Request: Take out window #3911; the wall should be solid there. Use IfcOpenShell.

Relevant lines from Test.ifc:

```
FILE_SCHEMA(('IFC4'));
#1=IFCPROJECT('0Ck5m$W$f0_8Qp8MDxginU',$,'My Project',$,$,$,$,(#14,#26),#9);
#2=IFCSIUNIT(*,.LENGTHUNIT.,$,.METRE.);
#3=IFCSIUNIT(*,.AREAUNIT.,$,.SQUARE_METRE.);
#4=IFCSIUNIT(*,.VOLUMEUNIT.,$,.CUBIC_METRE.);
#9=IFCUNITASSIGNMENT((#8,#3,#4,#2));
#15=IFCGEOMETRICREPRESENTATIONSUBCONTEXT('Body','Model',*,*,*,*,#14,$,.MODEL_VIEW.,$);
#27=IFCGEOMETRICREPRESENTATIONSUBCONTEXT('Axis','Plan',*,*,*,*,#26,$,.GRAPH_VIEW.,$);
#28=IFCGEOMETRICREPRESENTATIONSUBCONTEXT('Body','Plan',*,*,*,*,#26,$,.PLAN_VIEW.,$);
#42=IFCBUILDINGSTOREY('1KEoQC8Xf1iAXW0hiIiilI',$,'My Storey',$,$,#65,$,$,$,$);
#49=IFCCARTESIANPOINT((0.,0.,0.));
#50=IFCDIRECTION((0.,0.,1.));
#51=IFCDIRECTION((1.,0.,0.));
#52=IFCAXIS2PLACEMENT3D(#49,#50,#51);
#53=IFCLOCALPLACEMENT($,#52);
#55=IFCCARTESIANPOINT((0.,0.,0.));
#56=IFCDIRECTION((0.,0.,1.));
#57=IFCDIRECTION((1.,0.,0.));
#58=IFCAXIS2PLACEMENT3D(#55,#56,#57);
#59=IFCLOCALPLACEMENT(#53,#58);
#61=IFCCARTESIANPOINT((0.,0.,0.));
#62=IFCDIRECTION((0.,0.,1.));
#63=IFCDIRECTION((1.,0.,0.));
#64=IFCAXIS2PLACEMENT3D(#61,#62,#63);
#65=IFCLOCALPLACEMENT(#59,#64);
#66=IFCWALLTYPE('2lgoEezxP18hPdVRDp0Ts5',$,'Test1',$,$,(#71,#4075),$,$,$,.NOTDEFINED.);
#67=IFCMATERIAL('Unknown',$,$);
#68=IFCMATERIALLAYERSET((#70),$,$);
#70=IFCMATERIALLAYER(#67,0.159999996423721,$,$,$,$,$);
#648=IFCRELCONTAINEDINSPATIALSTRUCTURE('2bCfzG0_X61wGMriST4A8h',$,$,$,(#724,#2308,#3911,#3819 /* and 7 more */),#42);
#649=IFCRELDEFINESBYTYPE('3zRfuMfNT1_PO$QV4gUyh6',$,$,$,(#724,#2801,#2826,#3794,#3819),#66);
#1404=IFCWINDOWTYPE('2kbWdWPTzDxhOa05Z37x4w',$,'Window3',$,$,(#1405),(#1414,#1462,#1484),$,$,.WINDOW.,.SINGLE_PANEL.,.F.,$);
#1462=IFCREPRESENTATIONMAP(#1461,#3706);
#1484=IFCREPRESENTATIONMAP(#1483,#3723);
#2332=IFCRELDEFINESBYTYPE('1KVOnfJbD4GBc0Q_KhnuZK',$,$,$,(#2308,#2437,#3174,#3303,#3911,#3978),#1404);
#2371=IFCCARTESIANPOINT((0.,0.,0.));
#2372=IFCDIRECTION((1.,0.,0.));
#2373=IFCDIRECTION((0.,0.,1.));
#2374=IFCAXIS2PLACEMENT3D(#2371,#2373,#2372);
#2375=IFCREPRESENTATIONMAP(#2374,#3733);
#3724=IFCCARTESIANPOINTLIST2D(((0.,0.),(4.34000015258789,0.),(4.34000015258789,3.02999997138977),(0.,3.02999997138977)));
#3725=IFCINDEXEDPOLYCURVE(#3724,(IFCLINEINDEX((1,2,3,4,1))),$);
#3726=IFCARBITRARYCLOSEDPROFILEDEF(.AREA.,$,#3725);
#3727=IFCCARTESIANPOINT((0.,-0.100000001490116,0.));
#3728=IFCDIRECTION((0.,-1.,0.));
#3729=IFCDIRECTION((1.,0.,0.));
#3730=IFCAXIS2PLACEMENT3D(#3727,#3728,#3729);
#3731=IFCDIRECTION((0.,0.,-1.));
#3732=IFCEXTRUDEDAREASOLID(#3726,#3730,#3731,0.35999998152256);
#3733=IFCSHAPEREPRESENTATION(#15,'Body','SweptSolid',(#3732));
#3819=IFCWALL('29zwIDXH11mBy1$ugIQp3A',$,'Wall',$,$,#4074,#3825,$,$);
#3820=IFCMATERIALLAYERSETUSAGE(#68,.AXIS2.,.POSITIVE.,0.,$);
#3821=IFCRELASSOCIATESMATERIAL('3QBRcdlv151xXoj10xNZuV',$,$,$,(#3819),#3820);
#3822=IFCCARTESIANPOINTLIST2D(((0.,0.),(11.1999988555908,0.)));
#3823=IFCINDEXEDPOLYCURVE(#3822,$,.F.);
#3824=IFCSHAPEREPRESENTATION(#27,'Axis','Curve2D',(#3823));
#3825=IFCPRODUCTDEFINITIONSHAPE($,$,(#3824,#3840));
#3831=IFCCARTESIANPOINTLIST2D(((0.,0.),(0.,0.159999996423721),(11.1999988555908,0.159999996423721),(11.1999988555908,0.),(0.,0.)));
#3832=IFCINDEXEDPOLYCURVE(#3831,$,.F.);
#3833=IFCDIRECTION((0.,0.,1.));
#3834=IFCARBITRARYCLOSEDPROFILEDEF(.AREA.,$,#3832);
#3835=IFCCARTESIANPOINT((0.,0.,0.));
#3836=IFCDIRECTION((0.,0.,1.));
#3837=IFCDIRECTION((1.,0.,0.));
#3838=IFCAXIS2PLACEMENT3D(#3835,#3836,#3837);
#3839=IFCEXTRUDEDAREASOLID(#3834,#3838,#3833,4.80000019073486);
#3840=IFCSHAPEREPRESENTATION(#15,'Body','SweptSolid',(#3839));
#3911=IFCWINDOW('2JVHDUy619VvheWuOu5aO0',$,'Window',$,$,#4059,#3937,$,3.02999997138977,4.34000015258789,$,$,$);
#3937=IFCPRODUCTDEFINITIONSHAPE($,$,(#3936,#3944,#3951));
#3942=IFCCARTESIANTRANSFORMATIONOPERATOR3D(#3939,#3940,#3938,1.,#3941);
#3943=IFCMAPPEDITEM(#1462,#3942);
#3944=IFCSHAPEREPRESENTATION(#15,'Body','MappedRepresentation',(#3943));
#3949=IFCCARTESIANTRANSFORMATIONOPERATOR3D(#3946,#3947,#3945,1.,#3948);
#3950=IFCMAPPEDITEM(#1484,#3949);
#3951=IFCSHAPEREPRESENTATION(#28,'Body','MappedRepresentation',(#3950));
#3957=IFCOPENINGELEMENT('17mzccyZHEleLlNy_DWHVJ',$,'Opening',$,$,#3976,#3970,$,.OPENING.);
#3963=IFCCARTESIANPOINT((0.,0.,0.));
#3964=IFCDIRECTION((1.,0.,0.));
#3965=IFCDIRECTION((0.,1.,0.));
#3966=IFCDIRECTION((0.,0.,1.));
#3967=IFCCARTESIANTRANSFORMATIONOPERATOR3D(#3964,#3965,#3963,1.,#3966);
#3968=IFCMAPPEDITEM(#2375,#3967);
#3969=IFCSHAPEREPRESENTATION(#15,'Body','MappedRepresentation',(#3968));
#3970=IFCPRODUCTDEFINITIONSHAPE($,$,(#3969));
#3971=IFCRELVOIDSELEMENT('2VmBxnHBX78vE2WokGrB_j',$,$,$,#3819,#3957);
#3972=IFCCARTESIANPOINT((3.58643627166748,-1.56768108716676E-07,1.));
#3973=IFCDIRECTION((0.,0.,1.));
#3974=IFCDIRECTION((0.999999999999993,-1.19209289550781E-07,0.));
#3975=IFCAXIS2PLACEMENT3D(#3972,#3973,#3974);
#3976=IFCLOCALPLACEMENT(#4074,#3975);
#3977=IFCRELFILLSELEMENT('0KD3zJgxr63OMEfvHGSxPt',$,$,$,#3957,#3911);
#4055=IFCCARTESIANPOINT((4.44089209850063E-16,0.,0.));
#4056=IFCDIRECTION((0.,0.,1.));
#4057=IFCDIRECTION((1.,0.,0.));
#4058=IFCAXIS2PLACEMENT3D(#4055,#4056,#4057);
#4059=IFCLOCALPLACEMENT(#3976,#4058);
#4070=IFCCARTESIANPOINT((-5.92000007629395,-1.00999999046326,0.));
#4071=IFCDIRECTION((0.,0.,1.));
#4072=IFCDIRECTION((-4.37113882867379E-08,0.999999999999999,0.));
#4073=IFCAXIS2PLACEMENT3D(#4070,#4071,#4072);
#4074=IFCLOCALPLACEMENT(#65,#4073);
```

```python
import ifcopenshell
import ifcopenshell.api.feature
import ifcopenshell.api.root
import ifcopenshell.geom
import ifcopenshell.util.shape

model = ifcopenshell.open("Test.ifc")
settings = ifcopenshell.geom.settings()


def volume(element):
    """Net volume in cubic metres, openings subtracted."""
    shape = ifcopenshell.geom.create_shape(settings, element)
    return ifcopenshell.util.shape.get_volume(shape.geometry)


window = model.by_guid("2JVHDUy619VvheWuOu5aO0")
opening = window.FillsVoids[0].RelatingOpeningElement
wall = opening.VoidsElements[0].RelatingBuildingElement
before = volume(wall)

ifcopenshell.api.root.remove_product(model, product=window)
ifcopenshell.api.feature.remove_feature(model, feature=opening)

after = volume(wall)

print(f"wall volume {before:.3f} -> {after:.3f} m3")

model.write("Test_v2.ifc")
```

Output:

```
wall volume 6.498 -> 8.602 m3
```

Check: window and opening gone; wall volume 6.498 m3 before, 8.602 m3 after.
